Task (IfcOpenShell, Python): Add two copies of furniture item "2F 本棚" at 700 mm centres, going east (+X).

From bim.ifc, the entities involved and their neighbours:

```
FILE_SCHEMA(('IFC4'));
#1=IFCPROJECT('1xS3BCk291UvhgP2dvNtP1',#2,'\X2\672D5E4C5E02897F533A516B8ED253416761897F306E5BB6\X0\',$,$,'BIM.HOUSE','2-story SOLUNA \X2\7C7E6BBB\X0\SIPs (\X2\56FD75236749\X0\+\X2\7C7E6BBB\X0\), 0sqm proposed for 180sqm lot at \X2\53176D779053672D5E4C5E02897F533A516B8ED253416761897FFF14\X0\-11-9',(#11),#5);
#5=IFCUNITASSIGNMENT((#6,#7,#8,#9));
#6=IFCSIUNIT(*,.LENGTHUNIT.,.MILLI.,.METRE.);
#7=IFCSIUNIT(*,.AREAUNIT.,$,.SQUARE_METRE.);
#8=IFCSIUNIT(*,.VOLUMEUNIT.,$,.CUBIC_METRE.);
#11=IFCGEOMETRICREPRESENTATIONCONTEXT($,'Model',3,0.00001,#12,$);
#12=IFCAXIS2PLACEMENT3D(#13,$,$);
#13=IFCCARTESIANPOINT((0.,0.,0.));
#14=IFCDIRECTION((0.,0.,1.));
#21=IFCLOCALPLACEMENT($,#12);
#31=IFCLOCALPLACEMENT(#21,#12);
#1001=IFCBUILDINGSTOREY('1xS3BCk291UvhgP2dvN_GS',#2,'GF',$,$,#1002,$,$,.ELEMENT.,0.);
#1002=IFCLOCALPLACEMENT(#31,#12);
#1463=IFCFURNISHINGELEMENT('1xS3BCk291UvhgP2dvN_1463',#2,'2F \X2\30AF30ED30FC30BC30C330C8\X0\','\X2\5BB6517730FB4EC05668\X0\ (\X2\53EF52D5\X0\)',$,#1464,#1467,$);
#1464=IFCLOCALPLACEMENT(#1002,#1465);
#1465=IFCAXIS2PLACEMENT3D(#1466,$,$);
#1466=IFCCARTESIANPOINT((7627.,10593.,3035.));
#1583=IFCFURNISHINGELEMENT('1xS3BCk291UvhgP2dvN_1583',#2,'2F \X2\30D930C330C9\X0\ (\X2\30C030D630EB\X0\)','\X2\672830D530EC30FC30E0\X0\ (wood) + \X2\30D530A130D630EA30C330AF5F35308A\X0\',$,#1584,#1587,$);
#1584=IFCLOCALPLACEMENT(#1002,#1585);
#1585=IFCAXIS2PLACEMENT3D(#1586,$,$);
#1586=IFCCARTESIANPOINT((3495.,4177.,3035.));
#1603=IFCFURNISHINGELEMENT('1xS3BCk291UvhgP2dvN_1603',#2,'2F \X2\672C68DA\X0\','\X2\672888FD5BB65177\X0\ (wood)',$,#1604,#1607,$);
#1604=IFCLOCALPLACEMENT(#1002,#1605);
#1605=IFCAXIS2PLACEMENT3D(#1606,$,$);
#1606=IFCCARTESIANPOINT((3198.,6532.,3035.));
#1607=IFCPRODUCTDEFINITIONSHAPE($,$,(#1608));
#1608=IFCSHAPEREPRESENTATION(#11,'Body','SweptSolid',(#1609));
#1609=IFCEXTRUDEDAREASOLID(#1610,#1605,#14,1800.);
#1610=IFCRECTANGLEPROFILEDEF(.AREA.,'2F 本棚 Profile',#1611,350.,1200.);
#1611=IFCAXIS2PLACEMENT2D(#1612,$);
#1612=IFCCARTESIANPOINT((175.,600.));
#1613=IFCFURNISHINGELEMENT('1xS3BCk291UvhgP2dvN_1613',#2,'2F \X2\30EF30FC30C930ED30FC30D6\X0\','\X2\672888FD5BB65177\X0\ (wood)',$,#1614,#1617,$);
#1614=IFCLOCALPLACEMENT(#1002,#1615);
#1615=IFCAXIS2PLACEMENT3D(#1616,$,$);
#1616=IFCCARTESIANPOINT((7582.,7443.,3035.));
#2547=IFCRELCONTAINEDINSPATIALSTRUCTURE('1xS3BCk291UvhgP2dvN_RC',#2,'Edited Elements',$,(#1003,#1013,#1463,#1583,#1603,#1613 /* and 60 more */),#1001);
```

```python
import numpy as np
import ifcopenshell
import ifcopenshell.api.geometry
import ifcopenshell.api.root
import ifcopenshell.util.element
import ifcopenshell.util.placement

model = ifcopenshell.open("bim.ifc")


def reuse_history(source, copy):
    """copy_class also copies each property set's owner history, people and application; keep the originals."""
    for rel in copy.IsDefinedBy:
        if rel.is_a("IfcRelDefinesByProperties") and (history := rel.RelatingPropertyDefinition.OwnerHistory):
            rel.RelatingPropertyDefinition.OwnerHistory = source.OwnerHistory
            ifcopenshell.util.element.remove_deep2(model, history)


source = model.by_guid("1xS3BCk291UvhgP2dvN_1603")
base = ifcopenshell.util.placement.get_local_placement(source.ObjectPlacement)
step = np.array([1.0, 0.0, 0.0]) * 700.0

for i in range(1, 3):
    copy = ifcopenshell.api.root.copy_class(model, product=source)
    copy.Representation = ifcopenshell.util.element.copy_deep(
        model, source.Representation, exclude=["IfcGeometricRepresentationContext", "IfcRepresentationMap"]
    )
    reuse_history(source, copy)
    matrix = base.copy()
    matrix[:3, 3] += i * step
    print("added at", matrix[:3, 3].round(3) + 0.0)
    ifcopenshell.api.geometry.edit_object_placement(model, product=copy, matrix=matrix, is_si=False)

model.write("bim_v2.ifc")
```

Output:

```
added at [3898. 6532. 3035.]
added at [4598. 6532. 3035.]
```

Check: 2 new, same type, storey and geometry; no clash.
